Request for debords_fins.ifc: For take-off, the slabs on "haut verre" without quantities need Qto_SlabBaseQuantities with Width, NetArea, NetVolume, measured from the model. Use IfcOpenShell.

First a look at what the model holds.

```python
import ifcopenshell
import ifcopenshell.util.element
import ifcopenshell.util.unit

model = ifcopenshell.open("debords_fins.ifc")
print(model.schema)
for unit_type in ("LENGTHUNIT", "AREAUNIT", "VOLUMEUNIT"):
    print(unit_type, ifcopenshell.util.unit.calculate_unit_scale(model, unit_type))
storey = next(s for s in model.by_type("IfcBuildingStorey") if s.Name == "haut verre")
slabs = [e for e in ifcopenshell.util.element.get_decomposition(storey) if e.is_a("IfcSlab")]
for e in sorted(slabs, key=lambda e: e.id()):
    print(e.id(), e.is_a(), e.Name, list(ifcopenshell.util.element.get_psets(e, qtos_only=True)), sep=" | ")
```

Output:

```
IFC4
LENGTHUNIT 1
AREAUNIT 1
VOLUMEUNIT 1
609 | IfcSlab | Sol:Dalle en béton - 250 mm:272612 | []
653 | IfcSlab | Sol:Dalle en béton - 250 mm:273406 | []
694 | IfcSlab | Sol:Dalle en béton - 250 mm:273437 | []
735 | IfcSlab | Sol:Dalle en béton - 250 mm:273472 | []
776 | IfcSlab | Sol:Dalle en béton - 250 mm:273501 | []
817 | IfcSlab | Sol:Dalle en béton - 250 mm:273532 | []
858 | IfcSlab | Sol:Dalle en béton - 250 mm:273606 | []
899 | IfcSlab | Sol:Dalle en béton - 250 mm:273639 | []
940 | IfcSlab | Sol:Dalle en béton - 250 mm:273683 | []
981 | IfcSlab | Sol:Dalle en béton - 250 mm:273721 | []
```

```python
import ifcopenshell
import ifcopenshell.api.pset
import ifcopenshell.geom
import ifcopenshell.util.element
import ifcopenshell.util.shape
import ifcopenshell.util.unit

model = ifcopenshell.open("debords_fins.ifc")
unit_scale = ifcopenshell.util.unit.calculate_unit_scale(model)
area_scale = ifcopenshell.util.unit.calculate_unit_scale(model, "AREAUNIT")
volume_scale = ifcopenshell.util.unit.calculate_unit_scale(model, "VOLUMEUNIT")
settings = ifcopenshell.geom.settings()

storey = next(s for s in model.by_type("IfcBuildingStorey") if s.Name == "haut verre")
slabs = [e for e in ifcopenshell.util.element.get_decomposition(storey) if e.is_a("IfcSlab")]

for e in sorted(slabs, key=lambda e: e.id()):
    if ifcopenshell.util.element.get_psets(e, qtos_only=True, should_inherit=False):
        continue
    # Geometry comes back in metres, in the element's own axes.
    shape = ifcopenshell.geom.create_shape(settings, e)
    values = {
        "Width": ifcopenshell.util.shape.get_z(shape.geometry) / unit_scale,
        "NetArea": ifcopenshell.util.shape.get_footprint_area(shape.geometry) / area_scale,
        "NetVolume": ifcopenshell.util.shape.get_volume(shape.geometry) / volume_scale,
    }
    qto = ifcopenshell.api.pset.add_qto(model, product=e, name="Qto_SlabBaseQuantities")
    ifcopenshell.api.pset.edit_qto(model, qto=qto, properties=values)
    print(e.id(), {k: round(v, 3) for k, v in values.items()})

model.write("debords_fins_updated.ifc")
```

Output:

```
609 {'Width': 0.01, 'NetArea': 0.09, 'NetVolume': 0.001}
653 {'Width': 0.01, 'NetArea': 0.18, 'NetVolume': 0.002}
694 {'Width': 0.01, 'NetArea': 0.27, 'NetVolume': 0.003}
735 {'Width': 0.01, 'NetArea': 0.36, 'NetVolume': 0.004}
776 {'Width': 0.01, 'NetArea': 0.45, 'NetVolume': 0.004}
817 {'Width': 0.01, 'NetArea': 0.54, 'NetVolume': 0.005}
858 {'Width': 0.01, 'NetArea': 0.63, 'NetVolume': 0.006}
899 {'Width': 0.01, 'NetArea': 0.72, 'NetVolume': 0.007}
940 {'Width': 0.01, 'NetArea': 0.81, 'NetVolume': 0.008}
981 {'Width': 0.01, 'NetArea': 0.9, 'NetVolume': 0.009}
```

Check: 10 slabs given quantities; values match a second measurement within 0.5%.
